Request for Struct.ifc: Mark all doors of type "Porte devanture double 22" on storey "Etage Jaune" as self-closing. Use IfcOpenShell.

First a look at what the model holds.

```python
import ifcopenshell
import ifcopenshell.util.element

model = ifcopenshell.open("Struct.ifc")
print(model.schema)
storey = next(s for s in model.by_type("IfcBuildingStorey") if s.Name == "Etage Jaune")
doors = [e for e in ifcopenshell.util.element.get_decomposition(storey) if e.is_a("IfcDoor")]
seen = {}
for e in doors:
    element_type = ifcopenshell.util.element.get_type(e)
    key = (element_type.Name if element_type != e and element_type else None, ifcopenshell.util.element.get_pset(e, "Pset_DoorCommon", "SelfClosing"))
    seen[key] = seen.get(key, 0) + 1
for (name, value), count in sorted(seen.items(), key=str):
    print(count, "x", name, "|", value)
```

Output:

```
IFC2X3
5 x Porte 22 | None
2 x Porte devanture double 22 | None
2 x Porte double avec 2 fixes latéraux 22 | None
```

```python
import ifcopenshell
import ifcopenshell.api.pset
import ifcopenshell.util.element

model = ifcopenshell.open("Struct.ifc")

storey = next(s for s in model.by_type("IfcBuildingStorey") if s.Name == "Etage Jaune")
doors = [e for e in ifcopenshell.util.element.get_decomposition(storey) if e.is_a("IfcDoor")]

count = 0
for e in doors:
    element_type = ifcopenshell.util.element.get_type(e)
    if element_type in (None, e) or element_type.Name != "Porte devanture double 22":
        continue
    # add_pset returns the element's existing set when there is one.
    pset = ifcopenshell.api.pset.add_pset(model, product=e, name="Pset_DoorCommon")
    ifcopenshell.api.pset.edit_pset(model, pset=pset, properties={"SelfClosing": True})
    count += 1

print(count, "doors updated")

model.write("Struct_edited.ifc")
```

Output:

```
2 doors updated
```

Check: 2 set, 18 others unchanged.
